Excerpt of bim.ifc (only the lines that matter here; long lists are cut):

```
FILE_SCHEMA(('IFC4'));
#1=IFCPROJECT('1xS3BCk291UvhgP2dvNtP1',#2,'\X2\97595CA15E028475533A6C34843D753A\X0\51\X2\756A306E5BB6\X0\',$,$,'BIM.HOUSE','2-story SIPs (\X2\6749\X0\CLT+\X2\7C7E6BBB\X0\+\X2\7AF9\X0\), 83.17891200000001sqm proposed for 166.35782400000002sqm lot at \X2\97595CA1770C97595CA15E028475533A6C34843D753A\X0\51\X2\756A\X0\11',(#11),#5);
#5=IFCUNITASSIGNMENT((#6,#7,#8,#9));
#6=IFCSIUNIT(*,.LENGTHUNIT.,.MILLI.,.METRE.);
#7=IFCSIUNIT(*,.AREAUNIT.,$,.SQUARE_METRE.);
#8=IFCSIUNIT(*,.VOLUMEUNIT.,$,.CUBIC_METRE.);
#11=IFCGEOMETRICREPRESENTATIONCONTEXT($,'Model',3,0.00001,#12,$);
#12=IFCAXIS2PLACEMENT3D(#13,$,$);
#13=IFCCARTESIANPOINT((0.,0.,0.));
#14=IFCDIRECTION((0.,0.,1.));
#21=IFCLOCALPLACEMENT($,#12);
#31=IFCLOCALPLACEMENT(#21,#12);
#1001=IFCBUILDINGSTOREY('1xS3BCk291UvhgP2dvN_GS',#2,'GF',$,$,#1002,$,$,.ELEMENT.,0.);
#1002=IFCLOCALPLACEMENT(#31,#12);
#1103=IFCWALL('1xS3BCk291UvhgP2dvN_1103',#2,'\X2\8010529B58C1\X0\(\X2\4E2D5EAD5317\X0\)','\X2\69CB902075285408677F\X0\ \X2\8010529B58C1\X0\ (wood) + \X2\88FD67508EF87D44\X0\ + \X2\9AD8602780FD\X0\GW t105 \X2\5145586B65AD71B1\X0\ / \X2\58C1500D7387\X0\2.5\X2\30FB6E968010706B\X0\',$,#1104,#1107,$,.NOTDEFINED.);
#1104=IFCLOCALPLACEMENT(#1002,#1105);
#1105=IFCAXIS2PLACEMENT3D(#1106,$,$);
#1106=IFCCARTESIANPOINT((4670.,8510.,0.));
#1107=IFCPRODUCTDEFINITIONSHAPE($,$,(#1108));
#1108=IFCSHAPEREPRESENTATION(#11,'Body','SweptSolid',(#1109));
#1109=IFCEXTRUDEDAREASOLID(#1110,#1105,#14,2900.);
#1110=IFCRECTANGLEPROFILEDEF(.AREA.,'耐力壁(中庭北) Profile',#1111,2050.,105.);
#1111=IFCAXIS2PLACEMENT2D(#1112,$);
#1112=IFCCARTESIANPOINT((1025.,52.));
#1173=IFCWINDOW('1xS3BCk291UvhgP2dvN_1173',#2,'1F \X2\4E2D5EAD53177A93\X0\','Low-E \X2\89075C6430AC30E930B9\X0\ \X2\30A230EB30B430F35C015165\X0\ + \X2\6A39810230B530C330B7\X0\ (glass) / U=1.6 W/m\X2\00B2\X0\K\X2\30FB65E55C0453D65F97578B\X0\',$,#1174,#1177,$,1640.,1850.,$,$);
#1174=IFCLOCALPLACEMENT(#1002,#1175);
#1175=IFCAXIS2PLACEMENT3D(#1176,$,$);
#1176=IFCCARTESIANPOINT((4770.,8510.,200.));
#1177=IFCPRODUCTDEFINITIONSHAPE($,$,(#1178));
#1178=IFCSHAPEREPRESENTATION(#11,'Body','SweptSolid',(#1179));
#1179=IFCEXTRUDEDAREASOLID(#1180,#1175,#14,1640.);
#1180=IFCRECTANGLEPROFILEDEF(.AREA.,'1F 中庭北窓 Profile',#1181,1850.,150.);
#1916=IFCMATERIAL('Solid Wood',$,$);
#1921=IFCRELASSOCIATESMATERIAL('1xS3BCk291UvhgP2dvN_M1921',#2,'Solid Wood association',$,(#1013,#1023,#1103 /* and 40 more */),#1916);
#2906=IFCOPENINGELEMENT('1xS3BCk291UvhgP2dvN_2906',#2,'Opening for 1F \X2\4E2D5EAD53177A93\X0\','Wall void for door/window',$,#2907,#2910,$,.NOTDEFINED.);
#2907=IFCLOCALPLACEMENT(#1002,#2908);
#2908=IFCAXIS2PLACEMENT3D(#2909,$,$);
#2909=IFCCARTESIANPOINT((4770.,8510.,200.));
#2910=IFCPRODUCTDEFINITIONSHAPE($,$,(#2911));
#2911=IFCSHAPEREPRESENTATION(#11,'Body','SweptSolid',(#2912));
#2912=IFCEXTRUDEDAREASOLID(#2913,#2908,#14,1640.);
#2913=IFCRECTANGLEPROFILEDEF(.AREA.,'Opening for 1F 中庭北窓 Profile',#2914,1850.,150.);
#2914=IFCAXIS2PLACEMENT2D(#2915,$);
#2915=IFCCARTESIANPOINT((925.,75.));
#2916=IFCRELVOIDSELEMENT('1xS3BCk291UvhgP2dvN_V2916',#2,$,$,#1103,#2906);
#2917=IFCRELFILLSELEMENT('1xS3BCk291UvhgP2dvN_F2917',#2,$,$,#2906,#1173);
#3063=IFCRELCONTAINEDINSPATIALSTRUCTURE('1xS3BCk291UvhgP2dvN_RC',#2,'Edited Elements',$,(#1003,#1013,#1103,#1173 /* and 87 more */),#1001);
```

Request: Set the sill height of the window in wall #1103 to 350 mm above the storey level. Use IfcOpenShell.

```python
import numpy as np
import ifcopenshell
import ifcopenshell.api.geometry
import ifcopenshell.geom
import ifcopenshell.util.element
import ifcopenshell.util.placement
import ifcopenshell.util.shape
import ifcopenshell.util.unit

model = ifcopenshell.open("bim.ifc")
unit_scale = ifcopenshell.util.unit.calculate_unit_scale(model)

window = model.by_guid("1xS3BCk291UvhgP2dvN_1173")
opening = window.FillsVoids[0].RelatingOpeningElement
storey = ifcopenshell.util.element.get_container(window, ifc_class="IfcBuildingStorey")
level = ifcopenshell.util.placement.get_local_placement(storey.ObjectPlacement)[2, 3]

# The opening's origin need not be at the sill, so measure its lowest point.
shape = ifcopenshell.geom.create_shape(ifcopenshell.geom.settings(), opening)
bottom = ifcopenshell.util.shape.get_shape_bottom_elevation(shape, shape.geometry) / unit_scale
dz = level + 0.35 / unit_scale - bottom

shift = np.array([0.0, 0.0, dz])
# The window is not placed relative to its opening, so move both.
for product in (opening, window):
    matrix = ifcopenshell.util.placement.get_local_placement(product.ObjectPlacement)
    matrix[:3, 3] += shift
    ifcopenshell.api.geometry.edit_object_placement(model, product=product, matrix=matrix, is_si=False)

print(f"moved by {dz * unit_scale:+.3f} m")

model.write("bim_edited.ifc")
```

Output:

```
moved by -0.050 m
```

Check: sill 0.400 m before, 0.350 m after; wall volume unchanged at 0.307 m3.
